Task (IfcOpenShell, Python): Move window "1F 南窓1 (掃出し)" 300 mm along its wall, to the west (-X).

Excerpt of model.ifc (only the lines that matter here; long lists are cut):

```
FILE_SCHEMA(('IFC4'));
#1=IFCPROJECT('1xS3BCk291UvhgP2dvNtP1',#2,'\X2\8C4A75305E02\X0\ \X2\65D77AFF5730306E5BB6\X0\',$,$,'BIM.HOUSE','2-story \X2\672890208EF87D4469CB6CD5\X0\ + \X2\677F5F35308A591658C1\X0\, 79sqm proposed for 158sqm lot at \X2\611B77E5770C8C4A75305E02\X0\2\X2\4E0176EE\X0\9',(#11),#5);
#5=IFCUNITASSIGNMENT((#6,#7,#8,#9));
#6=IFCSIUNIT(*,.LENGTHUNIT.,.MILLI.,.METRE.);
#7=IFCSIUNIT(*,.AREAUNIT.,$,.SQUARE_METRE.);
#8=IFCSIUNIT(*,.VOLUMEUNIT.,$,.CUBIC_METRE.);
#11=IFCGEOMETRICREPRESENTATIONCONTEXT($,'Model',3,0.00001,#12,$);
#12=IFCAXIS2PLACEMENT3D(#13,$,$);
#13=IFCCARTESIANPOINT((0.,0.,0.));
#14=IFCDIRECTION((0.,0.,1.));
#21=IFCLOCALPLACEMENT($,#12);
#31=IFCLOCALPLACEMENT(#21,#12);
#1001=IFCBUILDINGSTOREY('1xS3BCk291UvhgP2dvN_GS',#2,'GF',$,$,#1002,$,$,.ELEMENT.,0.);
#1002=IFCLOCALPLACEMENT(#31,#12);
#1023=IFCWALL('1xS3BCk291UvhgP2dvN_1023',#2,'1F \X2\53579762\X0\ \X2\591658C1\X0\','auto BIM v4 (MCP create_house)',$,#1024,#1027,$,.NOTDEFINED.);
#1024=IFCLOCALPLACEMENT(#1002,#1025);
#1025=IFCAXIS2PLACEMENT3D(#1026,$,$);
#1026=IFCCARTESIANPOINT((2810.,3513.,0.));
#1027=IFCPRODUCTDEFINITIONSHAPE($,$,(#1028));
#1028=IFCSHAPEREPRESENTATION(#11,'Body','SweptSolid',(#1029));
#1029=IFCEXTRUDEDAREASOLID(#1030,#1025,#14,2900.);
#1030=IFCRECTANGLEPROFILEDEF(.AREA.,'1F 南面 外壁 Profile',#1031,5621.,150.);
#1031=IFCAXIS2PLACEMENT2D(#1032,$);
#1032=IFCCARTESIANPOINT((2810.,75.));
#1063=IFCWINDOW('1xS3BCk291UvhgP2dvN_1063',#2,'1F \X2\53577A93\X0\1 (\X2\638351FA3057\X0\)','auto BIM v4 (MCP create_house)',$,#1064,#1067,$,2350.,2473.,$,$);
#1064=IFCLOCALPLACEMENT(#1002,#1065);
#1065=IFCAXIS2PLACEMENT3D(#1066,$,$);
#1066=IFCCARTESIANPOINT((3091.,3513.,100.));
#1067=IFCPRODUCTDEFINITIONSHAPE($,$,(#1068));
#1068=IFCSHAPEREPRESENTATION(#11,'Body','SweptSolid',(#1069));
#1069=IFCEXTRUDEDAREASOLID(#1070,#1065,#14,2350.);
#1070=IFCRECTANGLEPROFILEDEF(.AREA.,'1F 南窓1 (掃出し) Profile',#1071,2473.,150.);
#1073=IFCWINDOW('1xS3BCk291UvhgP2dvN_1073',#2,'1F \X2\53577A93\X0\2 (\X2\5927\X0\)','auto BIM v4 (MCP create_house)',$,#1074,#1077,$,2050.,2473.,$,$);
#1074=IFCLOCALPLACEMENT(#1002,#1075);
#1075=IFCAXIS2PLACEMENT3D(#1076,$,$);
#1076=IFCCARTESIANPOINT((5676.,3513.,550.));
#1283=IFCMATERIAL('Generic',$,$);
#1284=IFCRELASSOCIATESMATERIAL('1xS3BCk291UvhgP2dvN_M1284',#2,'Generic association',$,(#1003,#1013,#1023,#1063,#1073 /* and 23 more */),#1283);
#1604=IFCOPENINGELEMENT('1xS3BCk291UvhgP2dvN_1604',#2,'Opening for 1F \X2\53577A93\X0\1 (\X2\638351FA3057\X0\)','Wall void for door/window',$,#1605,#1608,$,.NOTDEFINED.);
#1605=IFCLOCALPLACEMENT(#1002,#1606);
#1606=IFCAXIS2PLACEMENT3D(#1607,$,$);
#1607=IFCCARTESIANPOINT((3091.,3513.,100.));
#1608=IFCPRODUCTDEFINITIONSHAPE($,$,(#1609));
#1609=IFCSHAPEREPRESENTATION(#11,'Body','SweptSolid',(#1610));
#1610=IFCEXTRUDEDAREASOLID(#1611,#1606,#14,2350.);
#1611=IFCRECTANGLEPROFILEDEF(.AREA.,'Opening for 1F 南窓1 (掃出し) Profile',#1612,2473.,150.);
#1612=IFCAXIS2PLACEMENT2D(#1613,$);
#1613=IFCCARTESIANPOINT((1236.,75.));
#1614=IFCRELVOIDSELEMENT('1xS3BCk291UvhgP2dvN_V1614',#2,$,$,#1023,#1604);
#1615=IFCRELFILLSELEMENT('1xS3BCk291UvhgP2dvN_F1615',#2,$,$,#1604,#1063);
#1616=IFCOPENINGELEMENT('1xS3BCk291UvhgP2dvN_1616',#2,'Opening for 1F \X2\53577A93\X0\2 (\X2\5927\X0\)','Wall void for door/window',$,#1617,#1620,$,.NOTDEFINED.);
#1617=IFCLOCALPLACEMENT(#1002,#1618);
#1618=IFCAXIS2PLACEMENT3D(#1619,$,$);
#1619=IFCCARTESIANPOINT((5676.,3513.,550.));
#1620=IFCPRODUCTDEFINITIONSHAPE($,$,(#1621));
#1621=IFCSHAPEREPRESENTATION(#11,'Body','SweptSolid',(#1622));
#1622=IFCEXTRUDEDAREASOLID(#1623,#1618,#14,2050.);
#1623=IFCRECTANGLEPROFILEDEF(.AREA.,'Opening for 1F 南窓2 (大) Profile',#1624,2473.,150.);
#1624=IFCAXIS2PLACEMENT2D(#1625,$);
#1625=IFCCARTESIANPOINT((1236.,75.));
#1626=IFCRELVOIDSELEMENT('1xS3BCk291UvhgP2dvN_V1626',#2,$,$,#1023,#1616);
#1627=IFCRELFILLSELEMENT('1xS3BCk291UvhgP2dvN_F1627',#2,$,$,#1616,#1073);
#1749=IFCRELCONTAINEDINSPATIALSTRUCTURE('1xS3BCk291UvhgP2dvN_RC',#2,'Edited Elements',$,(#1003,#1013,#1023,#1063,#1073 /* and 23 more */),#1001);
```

```python
import ifcopenshell
import ifcopenshell.api.geometry
import ifcopenshell.util.placement
import ifcopenshell.util.unit

model = ifcopenshell.open("model.ifc")
unit_scale = ifcopenshell.util.unit.calculate_unit_scale(model)

window = model.by_guid("1xS3BCk291UvhgP2dvN_1063")
opening = window.FillsVoids[0].RelatingOpeningElement
wall = opening.VoidsElements[0].RelatingBuildingElement

wall_matrix = ifcopenshell.util.placement.get_local_placement(wall.ObjectPlacement)
shift = wall_matrix[:3, 0] * -0.3 / unit_scale
before = ifcopenshell.util.placement.get_local_placement(window.ObjectPlacement)[:3, 3].copy()

# The window is not placed relative to its opening, so move both.
for product in (opening, window):
    matrix = ifcopenshell.util.placement.get_local_placement(product.ObjectPlacement)
    matrix[:3, 3] += shift
    ifcopenshell.api.geometry.edit_object_placement(model, product=product, matrix=matrix, is_si=False)

after = ifcopenshell.util.placement.get_local_placement(window.ObjectPlacement)[:3, 3]
print("window moved by", (after - before).round(3) + 0.0)

model.write("model-out.ifc")
```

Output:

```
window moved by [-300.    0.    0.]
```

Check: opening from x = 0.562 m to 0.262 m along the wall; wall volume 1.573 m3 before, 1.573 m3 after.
